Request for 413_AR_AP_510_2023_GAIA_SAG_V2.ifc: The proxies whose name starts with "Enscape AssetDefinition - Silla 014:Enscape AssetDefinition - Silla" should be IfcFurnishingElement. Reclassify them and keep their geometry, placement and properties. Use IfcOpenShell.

First a look at what the model holds.

```python
import re

import ifcopenshell

model = ifcopenshell.open("413_AR_AP_510_2023_GAIA_SAG_V2.ifc")
print(model.schema)
seen = {}
for e in model.by_type("IfcBuildingElementProxy"):
    name = re.sub(r":\d+(:\d+)?$", "", e.Name or "")  # drop the element id that some exporters append
    seen[name] = seen.get(name, 0) + 1
for name, count in sorted(seen.items()):
    print(count, "x", name)
```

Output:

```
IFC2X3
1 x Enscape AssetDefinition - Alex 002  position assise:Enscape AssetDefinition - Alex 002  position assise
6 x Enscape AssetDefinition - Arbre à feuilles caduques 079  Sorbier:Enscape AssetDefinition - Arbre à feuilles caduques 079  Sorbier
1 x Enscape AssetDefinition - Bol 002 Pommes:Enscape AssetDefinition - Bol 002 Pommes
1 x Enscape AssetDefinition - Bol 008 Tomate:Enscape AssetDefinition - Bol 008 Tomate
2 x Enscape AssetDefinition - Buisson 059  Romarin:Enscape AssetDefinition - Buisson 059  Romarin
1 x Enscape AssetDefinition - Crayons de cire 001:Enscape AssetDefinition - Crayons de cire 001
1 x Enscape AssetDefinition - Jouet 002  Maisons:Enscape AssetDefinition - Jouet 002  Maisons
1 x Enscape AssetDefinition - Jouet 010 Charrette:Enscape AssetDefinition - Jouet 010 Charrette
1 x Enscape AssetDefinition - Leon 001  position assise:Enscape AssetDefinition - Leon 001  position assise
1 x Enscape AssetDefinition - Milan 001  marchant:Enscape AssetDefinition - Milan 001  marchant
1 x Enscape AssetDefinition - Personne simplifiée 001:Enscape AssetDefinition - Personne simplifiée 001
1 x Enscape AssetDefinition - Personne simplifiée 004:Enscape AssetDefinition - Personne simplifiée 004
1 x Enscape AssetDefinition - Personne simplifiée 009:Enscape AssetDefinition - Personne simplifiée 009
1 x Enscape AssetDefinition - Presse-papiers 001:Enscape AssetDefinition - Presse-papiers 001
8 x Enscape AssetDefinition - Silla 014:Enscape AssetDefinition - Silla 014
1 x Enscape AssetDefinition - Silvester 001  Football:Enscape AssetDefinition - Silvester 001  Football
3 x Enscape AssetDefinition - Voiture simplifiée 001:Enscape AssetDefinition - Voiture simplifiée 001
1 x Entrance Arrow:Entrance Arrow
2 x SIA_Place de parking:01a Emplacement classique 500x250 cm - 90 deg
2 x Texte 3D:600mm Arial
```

```python
import ifcopenshell
import ifcopenshell.api.root

model = ifcopenshell.open("413_AR_AP_510_2023_GAIA_SAG_V2.ifc")

proxies = [e.id() for e in model.by_type("IfcBuildingElementProxy") if (e.Name or "").startswith("Enscape AssetDefinition - Silla 014:Enscape AssetDefinition - Silla")]
for step_id in proxies:
    proxy = model.by_id(step_id)
    # Reclassifying a typed element also reclassifies its type and the type's other occurrences.
    if proxy.is_a("IfcBuildingElementProxy"):
        ifcopenshell.api.root.reassign_class(model, product=proxy, ifc_class="IfcFurnishingElement")

print(sum(model.by_id(i).is_a("IfcFurnishingElement") for i in proxies), "reclassified")

model.write("413_AR_AP_510_2023_GAIA_SAG_V2_updated.ifc")
```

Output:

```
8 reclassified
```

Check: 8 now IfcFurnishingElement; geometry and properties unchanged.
